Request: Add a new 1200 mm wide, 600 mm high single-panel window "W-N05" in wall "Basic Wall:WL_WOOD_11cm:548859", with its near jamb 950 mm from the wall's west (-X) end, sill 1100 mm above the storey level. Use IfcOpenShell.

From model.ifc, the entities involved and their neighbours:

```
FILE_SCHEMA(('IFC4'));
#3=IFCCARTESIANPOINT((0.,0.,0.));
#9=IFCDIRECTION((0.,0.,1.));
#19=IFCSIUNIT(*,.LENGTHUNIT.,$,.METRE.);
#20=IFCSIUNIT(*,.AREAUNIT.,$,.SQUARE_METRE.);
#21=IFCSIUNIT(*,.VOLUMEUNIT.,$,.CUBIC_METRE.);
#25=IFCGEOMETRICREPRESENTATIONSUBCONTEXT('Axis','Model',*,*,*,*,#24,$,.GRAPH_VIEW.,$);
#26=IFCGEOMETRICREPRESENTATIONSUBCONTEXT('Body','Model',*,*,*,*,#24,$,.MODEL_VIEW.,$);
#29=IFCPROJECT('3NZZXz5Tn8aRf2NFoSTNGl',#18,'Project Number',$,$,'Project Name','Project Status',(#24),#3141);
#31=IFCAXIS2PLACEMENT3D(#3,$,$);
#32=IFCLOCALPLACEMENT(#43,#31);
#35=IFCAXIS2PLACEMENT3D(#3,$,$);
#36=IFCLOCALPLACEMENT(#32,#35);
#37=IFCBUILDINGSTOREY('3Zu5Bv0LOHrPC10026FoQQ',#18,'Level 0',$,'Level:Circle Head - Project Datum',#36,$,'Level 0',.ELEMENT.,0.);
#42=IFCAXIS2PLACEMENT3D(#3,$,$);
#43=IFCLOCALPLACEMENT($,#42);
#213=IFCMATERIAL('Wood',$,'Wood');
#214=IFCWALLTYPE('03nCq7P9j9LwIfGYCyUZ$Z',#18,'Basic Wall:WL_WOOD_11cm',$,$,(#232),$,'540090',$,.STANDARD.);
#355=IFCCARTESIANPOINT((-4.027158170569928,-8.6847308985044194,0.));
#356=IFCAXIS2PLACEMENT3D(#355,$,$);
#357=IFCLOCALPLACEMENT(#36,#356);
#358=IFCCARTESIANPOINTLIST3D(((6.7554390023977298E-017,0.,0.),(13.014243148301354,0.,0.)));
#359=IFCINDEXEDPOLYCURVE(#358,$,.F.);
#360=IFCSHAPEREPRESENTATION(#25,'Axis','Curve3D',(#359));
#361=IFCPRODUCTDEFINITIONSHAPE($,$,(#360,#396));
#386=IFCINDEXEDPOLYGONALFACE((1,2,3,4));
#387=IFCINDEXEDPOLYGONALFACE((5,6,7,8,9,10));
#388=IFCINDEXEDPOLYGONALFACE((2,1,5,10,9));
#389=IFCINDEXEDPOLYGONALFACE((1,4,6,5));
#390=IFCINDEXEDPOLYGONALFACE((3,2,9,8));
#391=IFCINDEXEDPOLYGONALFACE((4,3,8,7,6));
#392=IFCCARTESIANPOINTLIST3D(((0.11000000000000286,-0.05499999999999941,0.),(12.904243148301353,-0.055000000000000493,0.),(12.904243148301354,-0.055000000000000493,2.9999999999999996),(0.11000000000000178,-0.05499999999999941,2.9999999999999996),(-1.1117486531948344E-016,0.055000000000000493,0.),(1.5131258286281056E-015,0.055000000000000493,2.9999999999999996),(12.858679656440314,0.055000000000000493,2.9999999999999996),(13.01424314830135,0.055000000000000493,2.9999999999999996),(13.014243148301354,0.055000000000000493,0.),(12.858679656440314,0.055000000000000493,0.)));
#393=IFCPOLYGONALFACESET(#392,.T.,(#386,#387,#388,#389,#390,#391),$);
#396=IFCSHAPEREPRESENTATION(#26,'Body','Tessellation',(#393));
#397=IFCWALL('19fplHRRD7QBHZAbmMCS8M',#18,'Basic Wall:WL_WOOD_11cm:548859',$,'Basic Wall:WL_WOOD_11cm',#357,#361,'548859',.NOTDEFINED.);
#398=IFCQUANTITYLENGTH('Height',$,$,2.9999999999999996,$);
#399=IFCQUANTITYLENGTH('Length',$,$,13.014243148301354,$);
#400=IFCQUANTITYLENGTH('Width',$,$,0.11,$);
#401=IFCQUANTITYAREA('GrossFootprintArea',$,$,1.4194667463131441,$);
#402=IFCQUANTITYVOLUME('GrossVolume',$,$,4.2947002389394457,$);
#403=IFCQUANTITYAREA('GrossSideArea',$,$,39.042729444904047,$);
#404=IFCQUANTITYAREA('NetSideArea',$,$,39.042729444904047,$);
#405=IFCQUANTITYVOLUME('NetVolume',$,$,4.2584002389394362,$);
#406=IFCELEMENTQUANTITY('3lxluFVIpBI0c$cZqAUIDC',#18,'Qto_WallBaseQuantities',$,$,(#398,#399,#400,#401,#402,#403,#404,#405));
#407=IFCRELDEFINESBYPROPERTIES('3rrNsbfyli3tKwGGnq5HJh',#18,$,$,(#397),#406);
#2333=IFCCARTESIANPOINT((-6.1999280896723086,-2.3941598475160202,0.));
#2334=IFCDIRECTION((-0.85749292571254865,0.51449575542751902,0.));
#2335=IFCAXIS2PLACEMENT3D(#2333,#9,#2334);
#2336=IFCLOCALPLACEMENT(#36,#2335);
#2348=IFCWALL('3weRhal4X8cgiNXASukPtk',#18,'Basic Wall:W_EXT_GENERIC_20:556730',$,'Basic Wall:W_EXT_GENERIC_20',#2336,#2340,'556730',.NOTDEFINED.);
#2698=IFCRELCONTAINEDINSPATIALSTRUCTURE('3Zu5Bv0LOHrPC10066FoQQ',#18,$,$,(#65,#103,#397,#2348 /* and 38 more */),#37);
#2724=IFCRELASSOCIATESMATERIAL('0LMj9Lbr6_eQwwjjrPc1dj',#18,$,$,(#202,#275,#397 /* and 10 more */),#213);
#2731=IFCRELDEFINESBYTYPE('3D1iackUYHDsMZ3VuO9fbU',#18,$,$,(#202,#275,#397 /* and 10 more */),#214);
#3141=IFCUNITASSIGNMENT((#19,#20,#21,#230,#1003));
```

```python
import numpy as np
import ifcopenshell
import ifcopenshell.api.feature
import ifcopenshell.api.geometry
import ifcopenshell.api.pset
import ifcopenshell.api.root
import ifcopenshell.api.spatial
import ifcopenshell.geom
import ifcopenshell.util.element
import ifcopenshell.util.placement
import ifcopenshell.util.representation
import ifcopenshell.util.shape
import ifcopenshell.util.unit

model = ifcopenshell.open("model.ifc")
unit_scale = ifcopenshell.util.unit.calculate_unit_scale(model)
area_scale = ifcopenshell.util.unit.calculate_unit_scale(model, "AREAUNIT")
volume_scale = ifcopenshell.util.unit.calculate_unit_scale(model, "VOLUMEUNIT")
settings = ifcopenshell.geom.settings()


def volume(element):
    """Net volume in cubic metres, openings subtracted."""
    shape = ifcopenshell.geom.create_shape(settings, element)
    return ifcopenshell.util.shape.get_volume(shape.geometry)


wall = model.by_id(397)
storey = ifcopenshell.util.element.get_container(wall, ifc_class="IfcBuildingStorey")
context = ifcopenshell.util.representation.get_context(model, "Model", "Body", "MODEL_VIEW")
before = volume(wall)

width, height, from_end, sill = 1.2, 0.6, 0.95, 1.1  # metres

# The wall runs along its own X axis, and the end named is its -X end.
wall_shape = ifcopenshell.geom.create_shape(settings, wall)
x, y, z = ifcopenshell.util.shape.get_vertices(wall_shape.geometry).T
start = x.min() + from_end
face, thickness = float(y.min()), float(y.max() - y.min())
wall_matrix = ifcopenshell.util.placement.get_local_placement(wall.ObjectPlacement)
level = ifcopenshell.util.placement.get_local_placement(storey.ObjectPlacement)[2, 3]


def in_wall(x, y):
    """Placement at x, y metres in the wall's axes, at sill height."""
    matrix = wall_matrix.copy()
    matrix[:, 3] = wall_matrix @ np.array([x / unit_scale, y / unit_scale, 0.0, 1.0])
    matrix[2, 3] = level + sill / unit_scale
    return matrix


# Opening: a box that overshoots both wall faces by 50 mm.
opening = ifcopenshell.api.root.create_entity(model, ifc_class="IfcOpeningElement", predefined_type="OPENING")
box = ifcopenshell.api.geometry.add_wall_representation(
    model, context=context, length=width, height=height, thickness=thickness + 0.1
)
ifcopenshell.api.geometry.assign_representation(model, product=opening, representation=box)
ifcopenshell.api.geometry.edit_object_placement(model, product=opening, matrix=in_wall(start, face - 0.05), is_si=False)
ifcopenshell.api.feature.add_feature(model, feature=opening, element=wall)

window = ifcopenshell.api.root.create_entity(model, ifc_class="IfcWindow", name="W-N05", predefined_type="WINDOW")
window.OverallWidth, window.OverallHeight = width / unit_scale, height / unit_scale
window.PartitioningType = "SINGLE_PANEL"
body = ifcopenshell.api.geometry.add_window_representation(
    model,
    context=context,
    overall_width=window.OverallWidth,
    overall_height=window.OverallHeight,
    partition_type="SINGLE_PANEL",
)
ifcopenshell.api.geometry.assign_representation(model, product=window, representation=body)
ifcopenshell.api.spatial.assign_container(model, products=[window], relating_structure=storey)
ifcopenshell.api.feature.add_filling(model, opening=opening, element=window)

# Centre the window in the wall's thickness.
ifcopenshell.api.geometry.edit_object_placement(model, product=window, matrix=in_wall(start, face), is_si=False)
window_shape = ifcopenshell.geom.create_shape(settings, window)
depth = ifcopenshell.util.shape.get_vertices(window_shape.geometry)[:, 1]
offset = face + thickness / 2 - (depth.min() + depth.max()) / 2
ifcopenshell.api.geometry.edit_object_placement(model, product=window, matrix=in_wall(start, offset), is_si=False)

after = volume(wall)

# Update the wall's stored quantities.
qto = model.by_id(ifcopenshell.util.element.get_pset(wall, "Qto_WallBaseQuantities", should_inherit=False)["id"])
ifcopenshell.api.pset.edit_qto(model, qto=qto, properties={
    "NetSideArea": after / thickness / area_scale,
    "NetVolume": after / volume_scale,
})

print(f"wall volume {before:.3f} -> {after:.3f} m3")

model.write("model_edited.ifc")
```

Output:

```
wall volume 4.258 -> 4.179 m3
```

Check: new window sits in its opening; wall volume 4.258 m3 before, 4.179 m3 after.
